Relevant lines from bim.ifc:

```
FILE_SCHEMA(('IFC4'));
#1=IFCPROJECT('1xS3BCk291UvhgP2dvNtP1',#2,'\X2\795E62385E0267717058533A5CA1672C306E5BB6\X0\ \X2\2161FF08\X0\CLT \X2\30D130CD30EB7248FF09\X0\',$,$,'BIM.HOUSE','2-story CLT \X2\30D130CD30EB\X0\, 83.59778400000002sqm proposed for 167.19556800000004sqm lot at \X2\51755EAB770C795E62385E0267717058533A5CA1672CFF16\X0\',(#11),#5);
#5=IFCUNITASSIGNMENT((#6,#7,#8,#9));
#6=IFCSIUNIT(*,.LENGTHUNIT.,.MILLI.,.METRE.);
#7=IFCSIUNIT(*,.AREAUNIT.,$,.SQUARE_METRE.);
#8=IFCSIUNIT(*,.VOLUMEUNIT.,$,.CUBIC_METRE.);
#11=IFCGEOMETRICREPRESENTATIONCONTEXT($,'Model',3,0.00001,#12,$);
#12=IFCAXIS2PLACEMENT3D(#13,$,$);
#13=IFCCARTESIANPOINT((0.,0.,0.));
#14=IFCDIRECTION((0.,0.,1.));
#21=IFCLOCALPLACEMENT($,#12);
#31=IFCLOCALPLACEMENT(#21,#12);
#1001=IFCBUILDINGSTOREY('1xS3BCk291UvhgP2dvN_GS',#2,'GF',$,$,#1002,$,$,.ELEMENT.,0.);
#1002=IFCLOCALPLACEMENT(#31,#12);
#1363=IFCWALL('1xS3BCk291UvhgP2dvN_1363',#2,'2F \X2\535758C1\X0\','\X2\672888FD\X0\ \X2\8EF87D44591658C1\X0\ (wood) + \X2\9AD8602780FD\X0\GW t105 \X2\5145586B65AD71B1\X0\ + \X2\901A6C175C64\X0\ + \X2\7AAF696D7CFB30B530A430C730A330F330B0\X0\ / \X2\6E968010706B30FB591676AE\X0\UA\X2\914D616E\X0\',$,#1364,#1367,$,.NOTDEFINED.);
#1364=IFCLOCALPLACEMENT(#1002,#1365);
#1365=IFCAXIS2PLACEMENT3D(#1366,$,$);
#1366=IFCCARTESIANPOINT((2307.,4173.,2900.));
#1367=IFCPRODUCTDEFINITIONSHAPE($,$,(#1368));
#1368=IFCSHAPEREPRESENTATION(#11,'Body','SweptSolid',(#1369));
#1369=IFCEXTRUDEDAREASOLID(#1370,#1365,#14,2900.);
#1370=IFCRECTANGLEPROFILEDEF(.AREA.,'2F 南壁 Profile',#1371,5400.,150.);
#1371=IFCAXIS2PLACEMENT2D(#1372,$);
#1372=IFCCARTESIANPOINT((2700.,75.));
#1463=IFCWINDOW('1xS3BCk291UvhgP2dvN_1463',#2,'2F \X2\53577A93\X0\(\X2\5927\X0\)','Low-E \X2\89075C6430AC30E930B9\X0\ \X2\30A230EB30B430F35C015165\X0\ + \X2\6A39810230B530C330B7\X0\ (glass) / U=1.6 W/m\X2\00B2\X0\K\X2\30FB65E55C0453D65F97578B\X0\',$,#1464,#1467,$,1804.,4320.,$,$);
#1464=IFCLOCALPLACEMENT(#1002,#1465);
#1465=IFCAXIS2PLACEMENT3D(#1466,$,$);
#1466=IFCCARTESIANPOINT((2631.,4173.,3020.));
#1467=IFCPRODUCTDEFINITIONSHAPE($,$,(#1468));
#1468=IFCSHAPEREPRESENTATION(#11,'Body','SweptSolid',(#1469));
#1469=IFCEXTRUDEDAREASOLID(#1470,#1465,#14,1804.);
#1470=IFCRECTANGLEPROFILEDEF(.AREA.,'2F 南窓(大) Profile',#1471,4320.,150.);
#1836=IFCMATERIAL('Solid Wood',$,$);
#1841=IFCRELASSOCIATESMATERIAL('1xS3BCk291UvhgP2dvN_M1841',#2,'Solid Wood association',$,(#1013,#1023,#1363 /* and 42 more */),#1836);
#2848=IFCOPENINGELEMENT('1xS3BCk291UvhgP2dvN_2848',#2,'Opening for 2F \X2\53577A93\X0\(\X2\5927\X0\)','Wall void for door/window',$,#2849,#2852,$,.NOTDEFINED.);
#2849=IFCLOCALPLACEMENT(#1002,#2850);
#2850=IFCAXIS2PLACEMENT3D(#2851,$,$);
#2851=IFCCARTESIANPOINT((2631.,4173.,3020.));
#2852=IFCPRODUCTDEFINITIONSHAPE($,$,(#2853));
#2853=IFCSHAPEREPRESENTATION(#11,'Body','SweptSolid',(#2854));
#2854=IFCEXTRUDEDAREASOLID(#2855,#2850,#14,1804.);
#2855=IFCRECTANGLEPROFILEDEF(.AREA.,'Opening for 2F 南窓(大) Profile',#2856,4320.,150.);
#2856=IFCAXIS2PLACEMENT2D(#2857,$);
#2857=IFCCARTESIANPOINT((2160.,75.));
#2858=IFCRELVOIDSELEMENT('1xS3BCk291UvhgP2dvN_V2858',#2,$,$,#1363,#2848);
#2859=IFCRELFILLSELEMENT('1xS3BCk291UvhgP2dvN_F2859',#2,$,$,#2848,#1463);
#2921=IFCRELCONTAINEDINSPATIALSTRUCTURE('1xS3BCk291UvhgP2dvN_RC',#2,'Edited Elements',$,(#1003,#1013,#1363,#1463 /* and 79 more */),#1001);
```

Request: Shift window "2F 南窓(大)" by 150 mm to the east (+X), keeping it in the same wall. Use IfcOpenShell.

```python
import ifcopenshell
import ifcopenshell.api.geometry
import ifcopenshell.util.placement

model = ifcopenshell.open("bim.ifc")

window = model.by_guid("1xS3BCk291UvhgP2dvN_1463")
opening = window.FillsVoids[0].RelatingOpeningElement
wall = opening.VoidsElements[0].RelatingBuildingElement

wall_matrix = ifcopenshell.util.placement.get_local_placement(wall.ObjectPlacement)
shift = wall_matrix[:3, 0] * 150.0
before = ifcopenshell.util.placement.get_local_placement(window.ObjectPlacement)[:3, 3].copy()

# The window is not placed relative to its opening, so move both.
for product in (opening, window):
    matrix = ifcopenshell.util.placement.get_local_placement(product.ObjectPlacement)
    matrix[:3, 3] += shift
    ifcopenshell.api.geometry.edit_object_placement(model, product=product, matrix=matrix, is_si=False)

after = ifcopenshell.util.placement.get_local_placement(window.ObjectPlacement)[:3, 3]
print("window moved by", (after - before).round(3) + 0.0)

model.write("bim_edited.ifc")
```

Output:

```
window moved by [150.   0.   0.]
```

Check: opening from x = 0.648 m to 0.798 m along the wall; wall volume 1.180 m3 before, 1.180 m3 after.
